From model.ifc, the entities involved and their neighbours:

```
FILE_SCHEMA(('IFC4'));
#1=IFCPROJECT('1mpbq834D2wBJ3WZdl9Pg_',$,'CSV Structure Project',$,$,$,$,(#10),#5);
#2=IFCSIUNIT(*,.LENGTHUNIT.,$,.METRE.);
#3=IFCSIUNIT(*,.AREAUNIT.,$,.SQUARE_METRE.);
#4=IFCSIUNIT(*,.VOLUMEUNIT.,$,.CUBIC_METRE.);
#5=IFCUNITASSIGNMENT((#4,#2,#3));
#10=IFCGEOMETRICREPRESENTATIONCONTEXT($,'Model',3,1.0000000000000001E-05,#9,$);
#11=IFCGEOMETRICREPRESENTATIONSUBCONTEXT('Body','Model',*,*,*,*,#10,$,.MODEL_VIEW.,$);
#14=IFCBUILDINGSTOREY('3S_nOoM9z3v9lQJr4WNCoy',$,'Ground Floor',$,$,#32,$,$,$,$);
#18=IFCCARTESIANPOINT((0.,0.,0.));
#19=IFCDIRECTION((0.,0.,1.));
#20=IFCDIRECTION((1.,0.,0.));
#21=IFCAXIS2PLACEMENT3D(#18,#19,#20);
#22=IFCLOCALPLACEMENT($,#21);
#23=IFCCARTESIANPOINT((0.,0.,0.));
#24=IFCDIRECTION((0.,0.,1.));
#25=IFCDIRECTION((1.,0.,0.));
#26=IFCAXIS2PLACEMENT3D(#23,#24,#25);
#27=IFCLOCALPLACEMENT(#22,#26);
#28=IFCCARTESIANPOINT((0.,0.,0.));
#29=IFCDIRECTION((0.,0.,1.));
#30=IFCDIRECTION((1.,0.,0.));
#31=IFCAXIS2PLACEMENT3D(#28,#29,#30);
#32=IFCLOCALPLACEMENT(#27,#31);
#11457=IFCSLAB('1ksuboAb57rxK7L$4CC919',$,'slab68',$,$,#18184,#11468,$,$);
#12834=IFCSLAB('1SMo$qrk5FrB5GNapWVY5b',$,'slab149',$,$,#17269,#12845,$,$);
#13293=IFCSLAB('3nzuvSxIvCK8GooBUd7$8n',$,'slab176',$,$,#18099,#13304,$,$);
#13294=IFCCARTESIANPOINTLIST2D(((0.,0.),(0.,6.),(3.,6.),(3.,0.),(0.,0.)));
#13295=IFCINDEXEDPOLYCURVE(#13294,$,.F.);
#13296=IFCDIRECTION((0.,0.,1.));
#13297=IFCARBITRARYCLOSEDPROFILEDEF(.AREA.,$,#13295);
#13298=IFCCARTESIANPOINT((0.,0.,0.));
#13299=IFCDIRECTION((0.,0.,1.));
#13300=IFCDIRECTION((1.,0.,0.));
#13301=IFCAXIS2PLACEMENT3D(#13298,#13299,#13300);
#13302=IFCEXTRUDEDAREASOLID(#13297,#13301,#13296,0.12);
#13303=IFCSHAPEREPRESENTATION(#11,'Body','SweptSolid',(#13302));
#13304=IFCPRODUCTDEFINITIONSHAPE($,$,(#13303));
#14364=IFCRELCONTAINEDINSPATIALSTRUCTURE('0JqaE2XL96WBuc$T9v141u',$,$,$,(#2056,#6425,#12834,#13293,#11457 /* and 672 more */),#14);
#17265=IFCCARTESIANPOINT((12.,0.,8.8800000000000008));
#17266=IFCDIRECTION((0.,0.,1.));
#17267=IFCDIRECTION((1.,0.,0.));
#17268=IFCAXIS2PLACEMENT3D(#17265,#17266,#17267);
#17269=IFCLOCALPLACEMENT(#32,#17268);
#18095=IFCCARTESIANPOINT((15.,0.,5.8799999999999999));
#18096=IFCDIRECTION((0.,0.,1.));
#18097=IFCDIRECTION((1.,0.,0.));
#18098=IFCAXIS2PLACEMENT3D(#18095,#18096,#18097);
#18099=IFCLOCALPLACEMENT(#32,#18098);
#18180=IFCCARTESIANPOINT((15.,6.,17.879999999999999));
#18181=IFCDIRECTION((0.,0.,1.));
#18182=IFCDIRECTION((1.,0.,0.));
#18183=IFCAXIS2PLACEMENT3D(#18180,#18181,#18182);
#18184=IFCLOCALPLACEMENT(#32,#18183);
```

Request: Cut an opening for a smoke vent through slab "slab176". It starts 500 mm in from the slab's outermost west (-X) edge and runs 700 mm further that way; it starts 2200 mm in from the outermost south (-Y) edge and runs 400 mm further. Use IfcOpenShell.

```python
import numpy as np
import ifcopenshell
import ifcopenshell.api.feature
import ifcopenshell.api.geometry
import ifcopenshell.api.root
import ifcopenshell.geom
import ifcopenshell.util.placement
import ifcopenshell.util.representation
import ifcopenshell.util.shape
import ifcopenshell.util.unit

model = ifcopenshell.open("model.ifc")
unit_scale = ifcopenshell.util.unit.calculate_unit_scale(model)
settings = ifcopenshell.geom.settings()


def volume(element):
    """Net volume in cubic metres, openings subtracted."""
    shape = ifcopenshell.geom.create_shape(settings, element)
    return ifcopenshell.util.shape.get_volume(shape.geometry)


slab = model.by_guid("3nzuvSxIvCK8GooBUd7$8n")
before = volume(slab)

# Extent in the slab's own axes, in metres. The edges named are its -X and -Y sides.
slab_shape = ifcopenshell.geom.create_shape(settings, slab)
vertices = ifcopenshell.util.shape.get_vertices(slab_shape.geometry)
x_min, y_min, bottom = vertices.min(axis=0)
top = vertices[:, 2].max()

opening = ifcopenshell.api.root.create_entity(model, ifc_class="IfcOpeningElement", name="Smoke vent opening", predefined_type="OPENING")
context = ifcopenshell.util.representation.get_context(model, "Model", "Body", "MODEL_VIEW")
width, depth = 0.7, 0.4
outline = [(0.0, 0.0), (width, 0.0), (width, depth), (0.0, depth), (0.0, 0.0)]
# Overshoot both faces by 50 mm so the cut is clean.
shape = ifcopenshell.api.geometry.add_slab_representation(
    model, context=context, depth=top - bottom + 0.1, polyline=outline
)
ifcopenshell.api.geometry.assign_representation(model, product=opening, representation=shape)

matrix = ifcopenshell.util.placement.get_local_placement(slab.ObjectPlacement)
matrix[:, 3] = matrix @ np.append(np.array([x_min + 0.5, y_min + 2.2, bottom - 0.05]) / unit_scale, 1.0)
ifcopenshell.api.geometry.edit_object_placement(model, product=opening, matrix=matrix, is_si=False)
ifcopenshell.api.feature.add_feature(model, feature=opening, element=slab)

after = volume(slab)

print(f"slab volume {before:.3f} -> {after:.3f} m3")

model.write("model_rev.ifc")
```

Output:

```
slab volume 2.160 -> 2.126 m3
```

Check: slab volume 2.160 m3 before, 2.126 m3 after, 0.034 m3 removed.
